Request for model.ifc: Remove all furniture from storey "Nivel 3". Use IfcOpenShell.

First a look at what the model holds.

```python
import ifcopenshell
import ifcopenshell.util.element

model = ifcopenshell.open("model.ifc")
print(model.schema)
storey = next(s for s in model.by_type("IfcBuildingStorey") if s.Name == "Nivel 3")
furniture = [e for e in ifcopenshell.util.element.get_decomposition(storey) if e.is_a("IfcFurnishingElement")]
seen = {}
for e in furniture:
    element_type = ifcopenshell.util.element.get_type(e)
    name = element_type.Name if element_type not in (None, e) else None
    seen[name] = seen.get(name, 0) + 1
for name, count in sorted(seen.items(), key=str):
    print(count, "x", name)
```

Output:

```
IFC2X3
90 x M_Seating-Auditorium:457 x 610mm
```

```python
import ifcopenshell
import ifcopenshell.api.root
import ifcopenshell.util.element

model = ifcopenshell.open("model.ifc")

storey = next(s for s in model.by_type("IfcBuildingStorey") if s.Name == "Nivel 3")
furniture = [e for e in ifcopenshell.util.element.get_decomposition(storey) if e.is_a("IfcFurnishingElement")]

for e in furniture:
    ifcopenshell.api.root.remove_product(model, product=e)
print(len(furniture), "removed")

model.write("model_rev.ifc")
```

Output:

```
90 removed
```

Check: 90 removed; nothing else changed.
